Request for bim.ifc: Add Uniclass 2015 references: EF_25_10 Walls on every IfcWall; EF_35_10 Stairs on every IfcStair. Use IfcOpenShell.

First a look at what the model holds.

```python
import ifcopenshell

model = ifcopenshell.open("bim.ifc")
print(model.schema)
print("classifications:", [c.Name for c in model.by_type("IfcClassification")])
for ifc_class in ("IfcDoor", "IfcRoof", "IfcStair", "IfcWall", "IfcWindow"):
    print(ifc_class, len(model.by_type(ifc_class)))
```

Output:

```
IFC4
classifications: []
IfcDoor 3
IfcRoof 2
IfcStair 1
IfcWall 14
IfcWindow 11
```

```python
import ifcopenshell
import ifcopenshell.api.classification

model = ifcopenshell.open("bim.ifc")

system = ifcopenshell.api.classification.add_classification(model, classification="Uniclass 2015")

codes = {
    "IfcWall": ("EF_25_10", "Walls"),
    "IfcStair": ("EF_35_10", "Stairs"),
}
for ifc_class, (code, name) in codes.items():
    products = model.by_type(ifc_class)
    ifcopenshell.api.classification.add_reference(
        model, products=products, classification=system, identification=code, name=name
    )
    print(code, len(products))

model.write("bim_v2.ifc")
```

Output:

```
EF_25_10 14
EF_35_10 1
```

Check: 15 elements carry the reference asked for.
